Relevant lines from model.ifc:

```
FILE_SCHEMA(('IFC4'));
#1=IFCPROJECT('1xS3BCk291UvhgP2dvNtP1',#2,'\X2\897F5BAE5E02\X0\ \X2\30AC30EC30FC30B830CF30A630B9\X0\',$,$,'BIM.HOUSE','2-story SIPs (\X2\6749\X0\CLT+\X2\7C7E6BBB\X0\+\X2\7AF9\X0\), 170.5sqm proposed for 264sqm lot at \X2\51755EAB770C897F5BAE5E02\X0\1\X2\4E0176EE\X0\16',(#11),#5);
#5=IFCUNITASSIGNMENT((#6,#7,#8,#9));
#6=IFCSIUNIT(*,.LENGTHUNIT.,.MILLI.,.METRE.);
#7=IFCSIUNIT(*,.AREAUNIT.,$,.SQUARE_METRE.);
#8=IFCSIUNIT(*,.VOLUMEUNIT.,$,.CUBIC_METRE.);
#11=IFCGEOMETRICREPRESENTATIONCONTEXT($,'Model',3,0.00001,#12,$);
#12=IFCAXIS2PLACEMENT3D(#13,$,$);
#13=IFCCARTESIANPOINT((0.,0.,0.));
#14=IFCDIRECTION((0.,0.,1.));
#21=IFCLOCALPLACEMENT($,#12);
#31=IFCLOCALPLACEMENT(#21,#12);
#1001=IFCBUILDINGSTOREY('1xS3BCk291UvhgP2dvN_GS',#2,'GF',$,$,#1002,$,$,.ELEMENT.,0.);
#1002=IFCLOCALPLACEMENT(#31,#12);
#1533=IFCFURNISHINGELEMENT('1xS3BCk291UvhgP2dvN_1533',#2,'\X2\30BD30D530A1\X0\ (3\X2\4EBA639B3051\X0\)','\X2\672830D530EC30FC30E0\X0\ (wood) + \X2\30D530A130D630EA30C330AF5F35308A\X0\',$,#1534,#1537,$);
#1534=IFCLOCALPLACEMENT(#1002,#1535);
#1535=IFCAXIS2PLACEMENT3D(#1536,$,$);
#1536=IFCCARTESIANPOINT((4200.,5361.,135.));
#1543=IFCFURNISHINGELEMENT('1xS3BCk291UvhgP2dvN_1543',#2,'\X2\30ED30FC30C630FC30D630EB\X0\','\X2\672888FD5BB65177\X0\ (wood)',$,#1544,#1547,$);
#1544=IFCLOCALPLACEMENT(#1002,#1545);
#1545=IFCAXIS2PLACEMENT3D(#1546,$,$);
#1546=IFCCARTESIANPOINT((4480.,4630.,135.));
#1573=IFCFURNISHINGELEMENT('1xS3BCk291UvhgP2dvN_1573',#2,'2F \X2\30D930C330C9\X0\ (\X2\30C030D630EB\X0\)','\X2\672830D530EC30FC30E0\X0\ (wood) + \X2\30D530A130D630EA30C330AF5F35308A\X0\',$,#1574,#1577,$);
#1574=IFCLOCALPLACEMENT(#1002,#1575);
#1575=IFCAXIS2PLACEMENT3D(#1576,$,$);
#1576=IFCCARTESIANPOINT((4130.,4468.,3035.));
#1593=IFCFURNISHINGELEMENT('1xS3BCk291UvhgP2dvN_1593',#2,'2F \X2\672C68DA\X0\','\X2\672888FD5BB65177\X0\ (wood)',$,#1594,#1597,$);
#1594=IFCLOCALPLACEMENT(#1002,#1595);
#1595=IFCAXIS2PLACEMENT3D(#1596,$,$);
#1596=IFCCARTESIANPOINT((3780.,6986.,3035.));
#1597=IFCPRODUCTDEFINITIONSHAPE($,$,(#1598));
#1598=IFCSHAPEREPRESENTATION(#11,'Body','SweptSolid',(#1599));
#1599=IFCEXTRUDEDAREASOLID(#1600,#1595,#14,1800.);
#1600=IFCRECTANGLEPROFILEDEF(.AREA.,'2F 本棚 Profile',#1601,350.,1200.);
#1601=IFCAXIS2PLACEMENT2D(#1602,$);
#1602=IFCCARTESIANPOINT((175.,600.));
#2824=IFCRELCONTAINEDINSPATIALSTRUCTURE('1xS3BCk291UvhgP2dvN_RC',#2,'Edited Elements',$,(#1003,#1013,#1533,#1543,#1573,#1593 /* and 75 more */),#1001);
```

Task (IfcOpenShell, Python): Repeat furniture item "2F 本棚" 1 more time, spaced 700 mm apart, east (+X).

```python
import numpy as np
import ifcopenshell
import ifcopenshell.api.geometry
import ifcopenshell.api.root
import ifcopenshell.util.element
import ifcopenshell.util.placement
import ifcopenshell.util.unit

model = ifcopenshell.open("model.ifc")
unit_scale = ifcopenshell.util.unit.calculate_unit_scale(model)


def reuse_history(source, copy):
    """copy_class also copies each property set's owner history, people and application; keep the originals."""
    for rel in copy.IsDefinedBy:
        if rel.is_a("IfcRelDefinesByProperties") and (history := rel.RelatingPropertyDefinition.OwnerHistory):
            rel.RelatingPropertyDefinition.OwnerHistory = source.OwnerHistory
            ifcopenshell.util.element.remove_deep2(model, history)


source = model.by_id(1593)
base = ifcopenshell.util.placement.get_local_placement(source.ObjectPlacement)
step = np.array([1.0, 0.0, 0.0]) * 0.7 / unit_scale

for i in range(1, 2):
    copy = ifcopenshell.api.root.copy_class(model, product=source)
    copy.Representation = ifcopenshell.util.element.copy_deep(
        model, source.Representation, exclude=["IfcGeometricRepresentationContext", "IfcRepresentationMap"]
    )
    reuse_history(source, copy)
    matrix = base.copy()
    matrix[:3, 3] += i * step
    print("added at", matrix[:3, 3].round(3) + 0.0)
    ifcopenshell.api.geometry.edit_object_placement(model, product=copy, matrix=matrix, is_si=False)

model.write("model_edited.ifc")
```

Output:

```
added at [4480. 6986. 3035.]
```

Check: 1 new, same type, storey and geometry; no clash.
